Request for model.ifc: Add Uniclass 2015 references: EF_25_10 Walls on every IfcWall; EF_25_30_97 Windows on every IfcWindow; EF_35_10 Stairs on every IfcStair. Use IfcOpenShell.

First a look at what the model holds.

```python
import ifcopenshell

model = ifcopenshell.open("model.ifc")
print(model.schema)
print("classifications:", [c.Name for c in model.by_type("IfcClassification")])
for ifc_class in ("IfcDoor", "IfcRoof", "IfcStair", "IfcWall", "IfcWindow"):
    print(ifc_class, len(model.by_type(ifc_class)))
```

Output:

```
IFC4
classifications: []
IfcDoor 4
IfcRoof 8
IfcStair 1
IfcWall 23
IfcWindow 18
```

```python
import ifcopenshell
import ifcopenshell.api.classification

model = ifcopenshell.open("model.ifc")

system = ifcopenshell.api.classification.add_classification(model, classification="Uniclass 2015")

codes = {
    "IfcWall": ("EF_25_10", "Walls"),
    "IfcWindow": ("EF_25_30_97", "Windows"),
    "IfcStair": ("EF_35_10", "Stairs"),
}
for ifc_class, (code, name) in codes.items():
    products = model.by_type(ifc_class)
    ifcopenshell.api.classification.add_reference(
        model, products=products, classification=system, identification=code, name=name
    )
    print(code, len(products))

model.write("model_rev.ifc")
```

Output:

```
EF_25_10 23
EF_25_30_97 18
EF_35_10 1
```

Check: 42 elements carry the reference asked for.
